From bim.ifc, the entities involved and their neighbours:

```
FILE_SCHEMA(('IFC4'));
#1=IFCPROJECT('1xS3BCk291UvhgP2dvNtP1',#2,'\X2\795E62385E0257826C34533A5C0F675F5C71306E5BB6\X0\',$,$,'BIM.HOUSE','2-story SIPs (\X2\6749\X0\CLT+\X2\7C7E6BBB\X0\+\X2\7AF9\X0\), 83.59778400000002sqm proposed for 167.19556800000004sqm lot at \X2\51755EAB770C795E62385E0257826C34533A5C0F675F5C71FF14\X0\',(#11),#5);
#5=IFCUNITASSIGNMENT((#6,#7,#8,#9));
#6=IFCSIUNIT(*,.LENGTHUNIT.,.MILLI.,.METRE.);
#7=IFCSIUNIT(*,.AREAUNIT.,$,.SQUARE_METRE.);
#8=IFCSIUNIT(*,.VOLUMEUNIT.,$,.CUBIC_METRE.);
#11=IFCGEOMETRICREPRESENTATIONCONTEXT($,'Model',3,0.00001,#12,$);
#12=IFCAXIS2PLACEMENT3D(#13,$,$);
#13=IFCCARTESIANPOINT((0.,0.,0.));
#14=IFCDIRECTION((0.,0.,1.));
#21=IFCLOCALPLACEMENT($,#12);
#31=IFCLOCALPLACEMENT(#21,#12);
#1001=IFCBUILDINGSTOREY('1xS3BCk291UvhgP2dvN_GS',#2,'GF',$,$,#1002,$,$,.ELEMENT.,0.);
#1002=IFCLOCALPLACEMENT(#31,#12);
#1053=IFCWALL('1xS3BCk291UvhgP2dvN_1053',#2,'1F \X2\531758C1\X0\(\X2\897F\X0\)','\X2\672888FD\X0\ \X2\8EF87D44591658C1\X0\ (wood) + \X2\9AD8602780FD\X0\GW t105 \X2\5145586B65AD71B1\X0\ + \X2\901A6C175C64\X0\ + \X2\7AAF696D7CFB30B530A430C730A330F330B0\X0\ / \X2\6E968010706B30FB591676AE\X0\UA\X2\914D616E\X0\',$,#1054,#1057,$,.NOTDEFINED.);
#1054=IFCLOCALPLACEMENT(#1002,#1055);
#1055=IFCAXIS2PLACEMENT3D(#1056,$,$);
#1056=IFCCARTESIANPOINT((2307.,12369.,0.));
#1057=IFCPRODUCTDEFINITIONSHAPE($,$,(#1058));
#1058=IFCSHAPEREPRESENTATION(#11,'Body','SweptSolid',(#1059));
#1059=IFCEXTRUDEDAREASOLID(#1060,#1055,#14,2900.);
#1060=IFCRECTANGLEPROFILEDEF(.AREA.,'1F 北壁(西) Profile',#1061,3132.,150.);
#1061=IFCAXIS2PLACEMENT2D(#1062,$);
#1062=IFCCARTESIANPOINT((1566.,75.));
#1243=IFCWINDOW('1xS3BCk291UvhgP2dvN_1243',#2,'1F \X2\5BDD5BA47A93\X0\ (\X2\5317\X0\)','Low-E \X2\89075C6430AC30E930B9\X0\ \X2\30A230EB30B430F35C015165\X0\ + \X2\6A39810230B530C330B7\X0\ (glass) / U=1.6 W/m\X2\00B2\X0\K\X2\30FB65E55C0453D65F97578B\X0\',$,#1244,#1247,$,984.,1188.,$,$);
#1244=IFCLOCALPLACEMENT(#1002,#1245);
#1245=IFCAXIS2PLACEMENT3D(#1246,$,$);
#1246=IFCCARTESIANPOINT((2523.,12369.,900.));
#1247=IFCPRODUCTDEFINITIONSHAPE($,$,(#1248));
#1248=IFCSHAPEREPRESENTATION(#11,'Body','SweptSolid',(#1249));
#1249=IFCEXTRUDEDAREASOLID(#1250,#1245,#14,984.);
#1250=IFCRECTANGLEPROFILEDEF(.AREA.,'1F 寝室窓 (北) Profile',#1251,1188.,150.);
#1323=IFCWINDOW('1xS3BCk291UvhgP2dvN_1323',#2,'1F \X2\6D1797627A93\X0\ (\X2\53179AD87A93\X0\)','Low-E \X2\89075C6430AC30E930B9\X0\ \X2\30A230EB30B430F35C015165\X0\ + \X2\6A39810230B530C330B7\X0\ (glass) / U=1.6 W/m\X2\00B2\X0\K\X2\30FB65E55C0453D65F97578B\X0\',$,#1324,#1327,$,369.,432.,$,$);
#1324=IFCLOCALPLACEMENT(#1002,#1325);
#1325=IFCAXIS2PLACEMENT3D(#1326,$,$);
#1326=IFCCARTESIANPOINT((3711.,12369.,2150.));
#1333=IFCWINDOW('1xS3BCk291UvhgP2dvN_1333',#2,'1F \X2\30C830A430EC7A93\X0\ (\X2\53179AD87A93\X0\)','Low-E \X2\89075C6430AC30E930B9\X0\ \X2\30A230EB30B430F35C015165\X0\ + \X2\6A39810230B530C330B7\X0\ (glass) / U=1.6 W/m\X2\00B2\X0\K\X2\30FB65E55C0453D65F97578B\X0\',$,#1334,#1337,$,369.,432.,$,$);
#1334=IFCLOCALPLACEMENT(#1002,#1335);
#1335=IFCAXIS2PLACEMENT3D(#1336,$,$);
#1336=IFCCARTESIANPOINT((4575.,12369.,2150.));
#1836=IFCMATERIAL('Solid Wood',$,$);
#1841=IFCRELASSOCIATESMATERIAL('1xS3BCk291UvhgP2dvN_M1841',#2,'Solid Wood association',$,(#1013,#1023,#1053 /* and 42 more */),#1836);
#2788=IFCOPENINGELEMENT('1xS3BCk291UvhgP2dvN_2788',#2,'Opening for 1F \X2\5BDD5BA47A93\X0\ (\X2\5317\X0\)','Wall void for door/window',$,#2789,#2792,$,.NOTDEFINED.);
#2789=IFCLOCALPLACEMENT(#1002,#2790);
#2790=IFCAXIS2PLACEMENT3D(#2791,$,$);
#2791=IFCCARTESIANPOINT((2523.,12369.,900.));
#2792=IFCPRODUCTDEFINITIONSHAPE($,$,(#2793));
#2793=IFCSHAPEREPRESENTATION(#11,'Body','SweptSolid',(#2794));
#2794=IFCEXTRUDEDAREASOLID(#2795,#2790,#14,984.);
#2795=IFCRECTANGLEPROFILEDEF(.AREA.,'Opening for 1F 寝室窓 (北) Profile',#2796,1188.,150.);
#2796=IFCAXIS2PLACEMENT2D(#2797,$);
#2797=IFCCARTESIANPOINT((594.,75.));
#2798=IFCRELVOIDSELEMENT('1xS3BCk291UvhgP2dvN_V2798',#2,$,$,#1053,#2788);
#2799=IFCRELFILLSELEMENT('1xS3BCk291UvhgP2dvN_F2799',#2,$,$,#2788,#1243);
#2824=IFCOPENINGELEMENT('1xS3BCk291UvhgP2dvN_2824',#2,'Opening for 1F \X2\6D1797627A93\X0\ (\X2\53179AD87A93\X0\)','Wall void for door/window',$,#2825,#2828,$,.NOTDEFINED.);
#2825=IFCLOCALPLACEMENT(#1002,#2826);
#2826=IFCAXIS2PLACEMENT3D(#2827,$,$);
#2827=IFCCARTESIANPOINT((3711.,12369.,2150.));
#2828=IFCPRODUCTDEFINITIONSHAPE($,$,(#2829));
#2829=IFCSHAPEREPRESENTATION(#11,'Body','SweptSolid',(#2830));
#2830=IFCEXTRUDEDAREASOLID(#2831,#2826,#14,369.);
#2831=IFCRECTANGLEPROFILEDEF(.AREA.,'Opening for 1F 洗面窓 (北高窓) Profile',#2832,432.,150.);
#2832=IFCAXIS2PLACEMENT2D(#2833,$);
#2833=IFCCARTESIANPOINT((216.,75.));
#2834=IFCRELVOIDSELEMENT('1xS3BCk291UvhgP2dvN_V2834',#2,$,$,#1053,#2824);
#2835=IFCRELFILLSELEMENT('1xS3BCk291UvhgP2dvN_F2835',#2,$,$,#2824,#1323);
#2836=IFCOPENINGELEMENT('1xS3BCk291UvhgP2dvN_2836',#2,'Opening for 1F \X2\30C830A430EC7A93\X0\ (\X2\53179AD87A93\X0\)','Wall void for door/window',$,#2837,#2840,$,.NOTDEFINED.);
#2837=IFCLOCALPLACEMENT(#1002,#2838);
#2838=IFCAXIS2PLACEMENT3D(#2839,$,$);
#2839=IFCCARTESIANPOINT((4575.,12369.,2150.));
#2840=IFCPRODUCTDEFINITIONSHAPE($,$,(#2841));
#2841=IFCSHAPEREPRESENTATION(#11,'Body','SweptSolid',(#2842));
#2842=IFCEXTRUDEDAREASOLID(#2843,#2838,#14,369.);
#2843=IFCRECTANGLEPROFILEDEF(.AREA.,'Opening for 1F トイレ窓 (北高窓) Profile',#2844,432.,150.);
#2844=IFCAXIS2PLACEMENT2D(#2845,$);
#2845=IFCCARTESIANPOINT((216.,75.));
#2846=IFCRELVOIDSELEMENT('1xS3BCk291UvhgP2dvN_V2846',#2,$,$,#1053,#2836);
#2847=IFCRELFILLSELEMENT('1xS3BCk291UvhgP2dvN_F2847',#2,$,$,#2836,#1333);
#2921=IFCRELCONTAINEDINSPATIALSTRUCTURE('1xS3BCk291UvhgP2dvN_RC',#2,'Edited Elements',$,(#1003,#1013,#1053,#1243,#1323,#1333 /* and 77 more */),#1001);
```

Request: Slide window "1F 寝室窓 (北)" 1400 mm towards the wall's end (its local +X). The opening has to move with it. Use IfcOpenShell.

```python
import ifcopenshell
import ifcopenshell.api.geometry
import ifcopenshell.util.placement
import ifcopenshell.util.unit

model = ifcopenshell.open("bim.ifc")
unit_scale = ifcopenshell.util.unit.calculate_unit_scale(model)

window = model.by_guid("1xS3BCk291UvhgP2dvN_1243")
opening = window.FillsVoids[0].RelatingOpeningElement
wall = opening.VoidsElements[0].RelatingBuildingElement

wall_matrix = ifcopenshell.util.placement.get_local_placement(wall.ObjectPlacement)
shift = wall_matrix[:3, 0] * 1.4 / unit_scale
before = ifcopenshell.util.placement.get_local_placement(window.ObjectPlacement)[:3, 3].copy()

# The window is not placed relative to its opening, so move both.
for product in (opening, window):
    matrix = ifcopenshell.util.placement.get_local_placement(product.ObjectPlacement)
    matrix[:3, 3] += shift
    ifcopenshell.api.geometry.edit_object_placement(model, product=product, matrix=matrix, is_si=False)

after = ifcopenshell.util.placement.get_local_placement(window.ObjectPlacement)[:3, 3]
print("window moved by", (after - before).round(3) + 0.0)

model.write("bim_updated.ifc")
```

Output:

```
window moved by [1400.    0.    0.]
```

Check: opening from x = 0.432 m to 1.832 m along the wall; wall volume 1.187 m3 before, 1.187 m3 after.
